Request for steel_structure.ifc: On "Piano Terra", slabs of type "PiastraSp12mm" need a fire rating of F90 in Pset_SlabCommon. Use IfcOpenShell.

First a look at what the model holds.

```python
import ifcopenshell
import ifcopenshell.util.element

model = ifcopenshell.open("steel_structure.ifc")
print(model.schema)
storey = next(s for s in model.by_type("IfcBuildingStorey") if s.Name == "Piano Terra")
slabs = [e for e in ifcopenshell.util.element.get_decomposition(storey) if e.is_a("IfcSlab")]
seen = {}
for e in slabs:
    element_type = ifcopenshell.util.element.get_type(e)
    key = (element_type.Name if element_type != e and element_type else None, ifcopenshell.util.element.get_pset(e, "Pset_SlabCommon", "FireRating"))
    seen[key] = seen.get(key, 0) + 1
for (name, value), count in sorted(seen.items(), key=str):
    print(count, "x", name, "|", value)
```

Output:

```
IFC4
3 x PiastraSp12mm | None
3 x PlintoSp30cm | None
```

```python
import ifcopenshell
import ifcopenshell.api.pset
import ifcopenshell.util.element

model = ifcopenshell.open("steel_structure.ifc")

storey = next(s for s in model.by_type("IfcBuildingStorey") if s.Name == "Piano Terra")
slabs = [e for e in ifcopenshell.util.element.get_decomposition(storey) if e.is_a("IfcSlab")]

count = 0
for e in slabs:
    element_type = ifcopenshell.util.element.get_type(e)
    if element_type in (None, e) or element_type.Name != "PiastraSp12mm":
        continue
    # add_pset returns the element's existing set when there is one.
    pset = ifcopenshell.api.pset.add_pset(model, product=e, name="Pset_SlabCommon")
    ifcopenshell.api.pset.edit_pset(model, pset=pset, properties={"FireRating": "F90"})
    count += 1

print(count, "slabs updated")

model.write("steel_structure_updated.ifc")
```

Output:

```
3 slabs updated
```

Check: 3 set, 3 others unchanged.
